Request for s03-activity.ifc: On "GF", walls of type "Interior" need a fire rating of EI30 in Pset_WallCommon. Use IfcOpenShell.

First a look at what the model holds.

```python
import ifcopenshell
import ifcopenshell.util.element

model = ifcopenshell.open("s03-activity.ifc")
print(model.schema)
storey = next(s for s in model.by_type("IfcBuildingStorey") if s.Name == "GF")
walls = [e for e in ifcopenshell.util.element.get_decomposition(storey) if e.is_a("IfcWall")]
seen = {}
for e in walls:
    element_type = ifcopenshell.util.element.get_type(e)
    key = (element_type.Name if element_type != e and element_type else None, ifcopenshell.util.element.get_pset(e, "Pset_WallCommon", "FireRating"))
    seen[key] = seen.get(key, 0) + 1
for (name, value), count in sorted(seen.items(), key=str):
    print(count, "x", name, "|", value)
```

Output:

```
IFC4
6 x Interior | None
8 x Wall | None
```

```python
import ifcopenshell
import ifcopenshell.api.pset
import ifcopenshell.util.element

model = ifcopenshell.open("s03-activity.ifc")

storey = next(s for s in model.by_type("IfcBuildingStorey") if s.Name == "GF")
walls = [e for e in ifcopenshell.util.element.get_decomposition(storey) if e.is_a("IfcWall")]

count = 0
for e in walls:
    element_type = ifcopenshell.util.element.get_type(e)
    if element_type in (None, e) or element_type.Name != "Interior":
        continue
    # add_pset returns the element's existing set when there is one.
    pset = ifcopenshell.api.pset.add_pset(model, product=e, name="Pset_WallCommon")
    ifcopenshell.api.pset.edit_pset(model, pset=pset, properties={"FireRating": "EI30"})
    count += 1

print(count, "walls updated")

model.write("s03-activity-out.ifc")
```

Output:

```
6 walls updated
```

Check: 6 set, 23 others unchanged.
